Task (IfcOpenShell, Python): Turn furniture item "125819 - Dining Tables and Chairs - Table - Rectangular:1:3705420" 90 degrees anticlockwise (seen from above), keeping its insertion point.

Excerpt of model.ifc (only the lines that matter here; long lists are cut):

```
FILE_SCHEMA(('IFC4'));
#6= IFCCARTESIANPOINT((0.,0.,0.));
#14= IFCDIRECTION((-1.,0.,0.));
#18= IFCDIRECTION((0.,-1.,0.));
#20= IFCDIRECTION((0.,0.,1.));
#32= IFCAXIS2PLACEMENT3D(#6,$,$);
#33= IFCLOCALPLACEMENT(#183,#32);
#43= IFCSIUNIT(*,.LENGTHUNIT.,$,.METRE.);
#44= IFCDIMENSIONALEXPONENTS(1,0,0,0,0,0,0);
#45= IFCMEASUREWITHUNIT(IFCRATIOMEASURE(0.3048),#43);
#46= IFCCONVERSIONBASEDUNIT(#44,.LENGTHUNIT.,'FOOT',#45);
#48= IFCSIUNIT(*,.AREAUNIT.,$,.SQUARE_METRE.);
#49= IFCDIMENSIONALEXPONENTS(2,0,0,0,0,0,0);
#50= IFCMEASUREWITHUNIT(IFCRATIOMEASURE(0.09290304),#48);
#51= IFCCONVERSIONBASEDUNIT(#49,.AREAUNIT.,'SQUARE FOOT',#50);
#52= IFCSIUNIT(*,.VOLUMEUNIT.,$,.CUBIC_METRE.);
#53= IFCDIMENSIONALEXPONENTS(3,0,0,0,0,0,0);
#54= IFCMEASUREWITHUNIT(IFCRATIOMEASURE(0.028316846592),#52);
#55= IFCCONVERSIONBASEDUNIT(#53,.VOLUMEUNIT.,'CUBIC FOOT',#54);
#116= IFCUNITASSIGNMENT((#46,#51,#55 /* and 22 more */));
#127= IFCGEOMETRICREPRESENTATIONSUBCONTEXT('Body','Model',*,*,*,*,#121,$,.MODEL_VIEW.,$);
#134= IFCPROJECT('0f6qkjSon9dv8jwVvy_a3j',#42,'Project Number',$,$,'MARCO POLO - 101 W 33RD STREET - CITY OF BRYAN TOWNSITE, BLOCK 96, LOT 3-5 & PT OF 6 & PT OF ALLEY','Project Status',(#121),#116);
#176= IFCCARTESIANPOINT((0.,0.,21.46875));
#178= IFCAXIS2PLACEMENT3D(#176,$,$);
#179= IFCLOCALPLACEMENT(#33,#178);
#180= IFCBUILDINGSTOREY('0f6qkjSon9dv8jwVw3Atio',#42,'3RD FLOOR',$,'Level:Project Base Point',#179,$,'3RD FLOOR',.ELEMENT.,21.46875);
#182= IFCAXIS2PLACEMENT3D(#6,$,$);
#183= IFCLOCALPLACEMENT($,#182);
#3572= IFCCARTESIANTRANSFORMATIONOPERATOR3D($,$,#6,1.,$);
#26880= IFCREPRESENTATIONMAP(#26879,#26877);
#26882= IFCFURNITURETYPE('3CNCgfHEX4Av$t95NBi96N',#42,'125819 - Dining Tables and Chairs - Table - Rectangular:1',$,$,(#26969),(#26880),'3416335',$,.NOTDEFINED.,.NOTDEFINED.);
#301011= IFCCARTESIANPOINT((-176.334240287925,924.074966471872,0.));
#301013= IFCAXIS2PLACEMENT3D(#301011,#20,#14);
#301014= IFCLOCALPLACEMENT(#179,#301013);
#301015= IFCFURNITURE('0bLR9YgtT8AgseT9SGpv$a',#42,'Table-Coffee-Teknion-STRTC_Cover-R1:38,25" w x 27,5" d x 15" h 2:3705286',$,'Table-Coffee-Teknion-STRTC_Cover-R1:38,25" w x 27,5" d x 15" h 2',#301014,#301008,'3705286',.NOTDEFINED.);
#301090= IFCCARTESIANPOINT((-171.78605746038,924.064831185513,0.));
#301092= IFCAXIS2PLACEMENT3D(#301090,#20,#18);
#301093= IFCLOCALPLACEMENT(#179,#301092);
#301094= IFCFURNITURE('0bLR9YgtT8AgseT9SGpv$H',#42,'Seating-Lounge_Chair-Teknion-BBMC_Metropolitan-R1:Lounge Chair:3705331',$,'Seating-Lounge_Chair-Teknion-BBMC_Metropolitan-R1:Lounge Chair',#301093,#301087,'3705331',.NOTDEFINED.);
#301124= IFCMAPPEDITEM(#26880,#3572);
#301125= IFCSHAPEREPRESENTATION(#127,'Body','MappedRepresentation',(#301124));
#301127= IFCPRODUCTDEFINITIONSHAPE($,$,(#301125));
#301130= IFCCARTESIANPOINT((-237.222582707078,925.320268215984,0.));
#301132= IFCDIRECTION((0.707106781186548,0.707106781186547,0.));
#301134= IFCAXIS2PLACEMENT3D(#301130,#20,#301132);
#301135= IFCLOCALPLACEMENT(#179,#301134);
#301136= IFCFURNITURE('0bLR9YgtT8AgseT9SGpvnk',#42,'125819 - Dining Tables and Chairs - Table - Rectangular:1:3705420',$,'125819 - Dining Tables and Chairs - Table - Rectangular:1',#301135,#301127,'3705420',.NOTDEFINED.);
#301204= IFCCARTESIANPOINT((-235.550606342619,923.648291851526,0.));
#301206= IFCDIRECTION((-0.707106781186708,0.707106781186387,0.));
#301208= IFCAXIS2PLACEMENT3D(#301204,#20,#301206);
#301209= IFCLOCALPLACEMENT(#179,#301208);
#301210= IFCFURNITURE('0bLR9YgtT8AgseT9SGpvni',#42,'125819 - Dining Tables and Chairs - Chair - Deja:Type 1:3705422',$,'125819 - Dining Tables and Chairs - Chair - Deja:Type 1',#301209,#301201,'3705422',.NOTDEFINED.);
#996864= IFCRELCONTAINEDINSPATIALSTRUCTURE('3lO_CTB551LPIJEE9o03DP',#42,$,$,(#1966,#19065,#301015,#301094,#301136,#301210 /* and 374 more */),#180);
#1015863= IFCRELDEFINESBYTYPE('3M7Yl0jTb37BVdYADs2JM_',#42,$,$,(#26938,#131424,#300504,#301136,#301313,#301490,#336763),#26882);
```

```python
import ifcopenshell
import ifcopenshell.api.geometry
import ifcopenshell.util.placement

model = ifcopenshell.open("model.ifc")

item = model.by_guid("0bLR9YgtT8AgseT9SGpvnk")
matrix = ifcopenshell.util.placement.get_local_placement(item.ObjectPlacement)
matrix = matrix @ ifcopenshell.util.placement.rotation(90, "Z")
ifcopenshell.api.geometry.edit_object_placement(model, product=item, matrix=matrix, is_si=False)

print(ifcopenshell.util.placement.get_local_placement(item.ObjectPlacement).round(3) + 0.0)

model.write("model_v2.ifc")
```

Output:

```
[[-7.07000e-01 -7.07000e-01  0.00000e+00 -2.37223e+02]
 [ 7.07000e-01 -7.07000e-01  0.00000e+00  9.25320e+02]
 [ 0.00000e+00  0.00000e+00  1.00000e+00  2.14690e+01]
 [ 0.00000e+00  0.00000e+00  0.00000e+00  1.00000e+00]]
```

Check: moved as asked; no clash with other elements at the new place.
